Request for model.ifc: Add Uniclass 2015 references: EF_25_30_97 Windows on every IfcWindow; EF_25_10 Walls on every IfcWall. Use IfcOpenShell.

First a look at what the model holds.

```python
import ifcopenshell

model = ifcopenshell.open("model.ifc")
print(model.schema)
print("classifications:", [c.Name for c in model.by_type("IfcClassification")])
for ifc_class in ("IfcDoor", "IfcRoof", "IfcStair", "IfcWall", "IfcWindow"):
    print(ifc_class, len(model.by_type(ifc_class)))
```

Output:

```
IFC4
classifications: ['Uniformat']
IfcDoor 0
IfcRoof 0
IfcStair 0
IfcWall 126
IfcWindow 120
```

```python
import ifcopenshell
import ifcopenshell.api.classification

model = ifcopenshell.open("model.ifc")

system = ifcopenshell.api.classification.add_classification(model, classification="Uniclass 2015")

codes = {
    "IfcWindow": ("EF_25_30_97", "Windows"),
    "IfcWall": ("EF_25_10", "Walls"),
}
for ifc_class, (code, name) in codes.items():
    products = model.by_type(ifc_class)
    ifcopenshell.api.classification.add_reference(
        model, products=products, classification=system, identification=code, name=name
    )
    print(code, len(products))

model.write("model-out.ifc")
```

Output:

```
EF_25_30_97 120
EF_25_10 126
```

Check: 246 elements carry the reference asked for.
